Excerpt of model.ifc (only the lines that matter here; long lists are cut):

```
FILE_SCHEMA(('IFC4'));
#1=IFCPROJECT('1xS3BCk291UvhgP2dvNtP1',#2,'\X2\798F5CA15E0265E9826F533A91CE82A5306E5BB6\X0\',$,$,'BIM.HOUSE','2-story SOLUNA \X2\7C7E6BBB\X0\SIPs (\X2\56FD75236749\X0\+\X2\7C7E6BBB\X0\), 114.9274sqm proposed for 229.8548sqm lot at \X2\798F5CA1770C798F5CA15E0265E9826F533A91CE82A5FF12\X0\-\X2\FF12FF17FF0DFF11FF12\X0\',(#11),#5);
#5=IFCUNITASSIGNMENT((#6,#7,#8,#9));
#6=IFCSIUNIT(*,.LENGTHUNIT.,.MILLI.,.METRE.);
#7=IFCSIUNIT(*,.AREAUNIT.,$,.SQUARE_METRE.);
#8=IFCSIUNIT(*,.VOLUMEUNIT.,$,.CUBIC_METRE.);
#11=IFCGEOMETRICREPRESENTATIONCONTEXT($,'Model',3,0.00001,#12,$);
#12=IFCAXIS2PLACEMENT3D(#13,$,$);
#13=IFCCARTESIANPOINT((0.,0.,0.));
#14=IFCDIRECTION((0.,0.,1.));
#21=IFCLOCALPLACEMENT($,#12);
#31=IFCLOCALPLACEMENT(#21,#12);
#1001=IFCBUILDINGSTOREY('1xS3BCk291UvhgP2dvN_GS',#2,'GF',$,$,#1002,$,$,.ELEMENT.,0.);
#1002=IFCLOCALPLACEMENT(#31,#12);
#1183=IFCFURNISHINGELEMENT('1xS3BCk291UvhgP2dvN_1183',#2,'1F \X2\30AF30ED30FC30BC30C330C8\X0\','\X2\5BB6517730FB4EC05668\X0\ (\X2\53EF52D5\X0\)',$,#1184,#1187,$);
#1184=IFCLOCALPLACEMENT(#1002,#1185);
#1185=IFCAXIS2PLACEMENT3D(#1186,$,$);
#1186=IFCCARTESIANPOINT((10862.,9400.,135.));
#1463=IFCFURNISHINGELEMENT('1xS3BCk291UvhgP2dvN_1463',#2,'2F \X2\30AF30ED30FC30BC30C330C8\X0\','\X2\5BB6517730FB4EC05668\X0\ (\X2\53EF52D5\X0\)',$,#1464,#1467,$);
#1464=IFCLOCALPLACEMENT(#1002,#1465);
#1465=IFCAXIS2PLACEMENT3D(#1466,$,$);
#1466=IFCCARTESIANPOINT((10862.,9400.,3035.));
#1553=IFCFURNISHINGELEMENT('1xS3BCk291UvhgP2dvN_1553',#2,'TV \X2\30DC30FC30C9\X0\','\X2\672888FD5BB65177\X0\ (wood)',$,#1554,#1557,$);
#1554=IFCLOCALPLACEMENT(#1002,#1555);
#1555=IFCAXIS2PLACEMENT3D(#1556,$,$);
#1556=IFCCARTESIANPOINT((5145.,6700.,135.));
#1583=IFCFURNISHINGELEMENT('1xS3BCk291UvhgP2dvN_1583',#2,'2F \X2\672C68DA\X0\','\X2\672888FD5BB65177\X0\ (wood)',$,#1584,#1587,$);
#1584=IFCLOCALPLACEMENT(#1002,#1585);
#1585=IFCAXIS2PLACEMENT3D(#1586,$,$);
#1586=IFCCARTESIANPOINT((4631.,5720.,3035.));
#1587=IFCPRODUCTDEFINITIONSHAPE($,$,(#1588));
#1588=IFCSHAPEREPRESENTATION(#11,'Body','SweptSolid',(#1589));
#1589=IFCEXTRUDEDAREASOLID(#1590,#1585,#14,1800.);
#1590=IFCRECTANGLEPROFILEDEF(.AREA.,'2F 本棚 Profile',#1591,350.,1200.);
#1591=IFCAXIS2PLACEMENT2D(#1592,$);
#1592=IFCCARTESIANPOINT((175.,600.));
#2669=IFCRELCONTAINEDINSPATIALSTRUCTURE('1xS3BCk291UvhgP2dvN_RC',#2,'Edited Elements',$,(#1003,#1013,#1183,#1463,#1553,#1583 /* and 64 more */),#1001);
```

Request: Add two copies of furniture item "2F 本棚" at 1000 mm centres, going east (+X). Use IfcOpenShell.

```python
import numpy as np
import ifcopenshell
import ifcopenshell.api.geometry
import ifcopenshell.api.root
import ifcopenshell.util.element
import ifcopenshell.util.placement
import ifcopenshell.util.unit

model = ifcopenshell.open("model.ifc")
unit_scale = ifcopenshell.util.unit.calculate_unit_scale(model)


def reuse_history(source, copy):
    """copy_class also copies each property set's owner history, people and application; keep the originals."""
    for rel in copy.IsDefinedBy:
        if rel.is_a("IfcRelDefinesByProperties") and (history := rel.RelatingPropertyDefinition.OwnerHistory):
            rel.RelatingPropertyDefinition.OwnerHistory = source.OwnerHistory
            ifcopenshell.util.element.remove_deep2(model, history)


source = model.by_guid("1xS3BCk291UvhgP2dvN_1583")
base = ifcopenshell.util.placement.get_local_placement(source.ObjectPlacement)
step = np.array([1.0, 0.0, 0.0]) * 1 / unit_scale

for i in range(1, 3):
    copy = ifcopenshell.api.root.copy_class(model, product=source)
    copy.Representation = ifcopenshell.util.element.copy_deep(
        model, source.Representation, exclude=["IfcGeometricRepresentationContext", "IfcRepresentationMap"]
    )
    reuse_history(source, copy)
    matrix = base.copy()
    matrix[:3, 3] += i * step
    print("added at", matrix[:3, 3].round(3) + 0.0)
    ifcopenshell.api.geometry.edit_object_placement(model, product=copy, matrix=matrix, is_si=False)

model.write("model_updated.ifc")
```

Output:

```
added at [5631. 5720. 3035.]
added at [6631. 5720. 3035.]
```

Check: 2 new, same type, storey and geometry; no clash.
